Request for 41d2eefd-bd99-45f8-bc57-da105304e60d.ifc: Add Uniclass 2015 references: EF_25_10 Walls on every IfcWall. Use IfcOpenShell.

First a look at what the model holds.

```python
import ifcopenshell

model = ifcopenshell.open("41d2eefd-bd99-45f8-bc57-da105304e60d.ifc")
print(model.schema)
print("classifications:", [c.Name for c in model.by_type("IfcClassification")])
for ifc_class in ("IfcDoor", "IfcRoof", "IfcStair", "IfcWall", "IfcWindow"):
    print(ifc_class, len(model.by_type(ifc_class)))
```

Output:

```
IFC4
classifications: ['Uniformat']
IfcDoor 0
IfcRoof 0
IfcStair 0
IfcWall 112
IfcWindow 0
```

```python
import ifcopenshell
import ifcopenshell.api.classification

model = ifcopenshell.open("41d2eefd-bd99-45f8-bc57-da105304e60d.ifc")

system = ifcopenshell.api.classification.add_classification(model, classification="Uniclass 2015")

codes = {
    "IfcWall": ("EF_25_10", "Walls"),
}
for ifc_class, (code, name) in codes.items():
    products = model.by_type(ifc_class)
    ifcopenshell.api.classification.add_reference(
        model, products=products, classification=system, identification=code, name=name
    )
    print(code, len(products))

model.write("41d2eefd-bd99-45f8-bc57-da105304e60d-out.ifc")
```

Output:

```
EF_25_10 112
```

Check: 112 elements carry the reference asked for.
